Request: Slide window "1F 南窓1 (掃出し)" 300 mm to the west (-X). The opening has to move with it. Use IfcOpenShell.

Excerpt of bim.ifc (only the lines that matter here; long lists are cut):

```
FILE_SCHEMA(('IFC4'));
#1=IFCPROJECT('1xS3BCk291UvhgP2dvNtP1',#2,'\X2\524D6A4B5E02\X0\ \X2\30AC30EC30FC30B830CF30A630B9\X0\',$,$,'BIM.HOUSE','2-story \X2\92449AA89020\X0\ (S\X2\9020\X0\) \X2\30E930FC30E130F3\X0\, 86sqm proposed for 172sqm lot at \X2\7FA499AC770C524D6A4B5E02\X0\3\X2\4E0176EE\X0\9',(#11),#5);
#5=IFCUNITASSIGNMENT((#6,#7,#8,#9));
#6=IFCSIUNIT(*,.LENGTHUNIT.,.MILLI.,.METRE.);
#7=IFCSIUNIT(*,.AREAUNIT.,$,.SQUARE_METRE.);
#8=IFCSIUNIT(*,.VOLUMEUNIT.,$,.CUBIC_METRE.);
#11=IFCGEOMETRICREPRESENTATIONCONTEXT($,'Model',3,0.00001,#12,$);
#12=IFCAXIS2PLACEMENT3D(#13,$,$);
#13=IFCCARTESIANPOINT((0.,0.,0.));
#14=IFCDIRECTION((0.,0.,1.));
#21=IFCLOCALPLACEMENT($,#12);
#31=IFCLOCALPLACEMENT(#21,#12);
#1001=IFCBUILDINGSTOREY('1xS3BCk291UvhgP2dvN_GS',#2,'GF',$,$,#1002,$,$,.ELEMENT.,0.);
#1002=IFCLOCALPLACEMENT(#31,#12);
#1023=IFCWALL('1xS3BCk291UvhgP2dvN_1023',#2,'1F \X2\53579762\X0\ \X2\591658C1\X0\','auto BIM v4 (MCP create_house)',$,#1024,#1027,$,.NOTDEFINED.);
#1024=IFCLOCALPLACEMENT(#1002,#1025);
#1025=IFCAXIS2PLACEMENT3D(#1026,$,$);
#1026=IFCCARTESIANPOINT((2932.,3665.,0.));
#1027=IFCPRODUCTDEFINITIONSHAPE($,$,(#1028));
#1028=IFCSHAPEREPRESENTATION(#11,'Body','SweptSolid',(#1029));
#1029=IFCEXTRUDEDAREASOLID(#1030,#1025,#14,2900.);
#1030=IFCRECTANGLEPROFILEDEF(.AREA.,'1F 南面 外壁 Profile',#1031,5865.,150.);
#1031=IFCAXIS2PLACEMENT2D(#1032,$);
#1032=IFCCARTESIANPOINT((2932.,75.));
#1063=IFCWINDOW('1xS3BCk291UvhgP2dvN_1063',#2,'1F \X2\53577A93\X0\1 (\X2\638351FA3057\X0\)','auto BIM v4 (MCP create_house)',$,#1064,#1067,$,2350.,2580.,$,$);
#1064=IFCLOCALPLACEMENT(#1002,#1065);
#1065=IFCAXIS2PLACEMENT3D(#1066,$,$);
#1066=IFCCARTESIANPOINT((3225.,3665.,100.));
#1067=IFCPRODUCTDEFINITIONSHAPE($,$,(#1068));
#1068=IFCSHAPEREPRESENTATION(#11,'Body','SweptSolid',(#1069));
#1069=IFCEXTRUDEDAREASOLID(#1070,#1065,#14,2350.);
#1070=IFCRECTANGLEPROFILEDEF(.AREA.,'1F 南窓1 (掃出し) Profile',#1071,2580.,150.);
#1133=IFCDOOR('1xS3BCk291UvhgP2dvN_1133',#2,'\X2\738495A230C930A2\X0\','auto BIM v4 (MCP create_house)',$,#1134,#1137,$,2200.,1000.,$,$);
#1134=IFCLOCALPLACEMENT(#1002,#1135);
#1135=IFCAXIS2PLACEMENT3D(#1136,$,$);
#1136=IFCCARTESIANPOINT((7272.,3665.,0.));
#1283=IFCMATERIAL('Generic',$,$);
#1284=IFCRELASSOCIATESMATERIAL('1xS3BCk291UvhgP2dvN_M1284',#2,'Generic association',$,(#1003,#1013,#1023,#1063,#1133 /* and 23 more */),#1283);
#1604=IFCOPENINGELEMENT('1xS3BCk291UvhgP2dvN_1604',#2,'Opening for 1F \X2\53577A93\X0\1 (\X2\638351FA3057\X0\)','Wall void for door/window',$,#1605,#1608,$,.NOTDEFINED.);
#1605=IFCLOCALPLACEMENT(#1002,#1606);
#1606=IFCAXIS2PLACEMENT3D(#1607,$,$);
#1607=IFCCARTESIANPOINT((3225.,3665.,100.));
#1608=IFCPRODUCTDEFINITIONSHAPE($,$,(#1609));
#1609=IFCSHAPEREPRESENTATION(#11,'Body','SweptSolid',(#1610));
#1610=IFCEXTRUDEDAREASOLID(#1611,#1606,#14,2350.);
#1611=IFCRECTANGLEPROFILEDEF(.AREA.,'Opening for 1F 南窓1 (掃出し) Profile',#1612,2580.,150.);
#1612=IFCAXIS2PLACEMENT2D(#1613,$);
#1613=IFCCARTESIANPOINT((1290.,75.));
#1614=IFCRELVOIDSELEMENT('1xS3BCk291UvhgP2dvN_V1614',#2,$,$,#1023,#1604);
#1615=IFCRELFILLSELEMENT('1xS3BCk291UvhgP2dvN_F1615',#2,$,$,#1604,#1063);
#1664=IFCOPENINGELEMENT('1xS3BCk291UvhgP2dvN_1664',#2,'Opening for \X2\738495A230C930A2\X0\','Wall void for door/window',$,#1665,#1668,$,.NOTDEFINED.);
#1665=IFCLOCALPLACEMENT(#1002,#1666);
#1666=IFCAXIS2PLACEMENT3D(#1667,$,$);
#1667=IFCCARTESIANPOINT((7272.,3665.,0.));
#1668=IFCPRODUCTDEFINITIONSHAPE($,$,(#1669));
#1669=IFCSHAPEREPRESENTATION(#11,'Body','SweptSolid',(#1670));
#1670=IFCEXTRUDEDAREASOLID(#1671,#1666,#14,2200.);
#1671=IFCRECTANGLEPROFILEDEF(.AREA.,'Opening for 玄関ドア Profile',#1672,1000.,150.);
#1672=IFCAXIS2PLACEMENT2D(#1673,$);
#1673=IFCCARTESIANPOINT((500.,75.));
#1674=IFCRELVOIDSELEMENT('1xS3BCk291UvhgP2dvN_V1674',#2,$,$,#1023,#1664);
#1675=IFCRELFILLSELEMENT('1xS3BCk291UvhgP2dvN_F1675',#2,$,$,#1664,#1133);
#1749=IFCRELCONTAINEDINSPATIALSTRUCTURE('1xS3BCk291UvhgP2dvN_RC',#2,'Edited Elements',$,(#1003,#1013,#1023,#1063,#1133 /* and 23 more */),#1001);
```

```python
import ifcopenshell
import ifcopenshell.api.geometry
import ifcopenshell.util.placement

model = ifcopenshell.open("bim.ifc")

window = model.by_guid("1xS3BCk291UvhgP2dvN_1063")
opening = window.FillsVoids[0].RelatingOpeningElement
wall = opening.VoidsElements[0].RelatingBuildingElement

wall_matrix = ifcopenshell.util.placement.get_local_placement(wall.ObjectPlacement)
shift = wall_matrix[:3, 0] * -300.0
before = ifcopenshell.util.placement.get_local_placement(window.ObjectPlacement)[:3, 3].copy()

# The window is not placed relative to its opening, so move both.
for product in (opening, window):
    matrix = ifcopenshell.util.placement.get_local_placement(product.ObjectPlacement)
    matrix[:3, 3] += shift
    ifcopenshell.api.geometry.edit_object_placement(model, product=product, matrix=matrix, is_si=False)

after = ifcopenshell.util.placement.get_local_placement(window.ObjectPlacement)[:3, 3]
print("window moved by", (after - before).round(3) + 0.0)

model.write("bim_updated.ifc")
```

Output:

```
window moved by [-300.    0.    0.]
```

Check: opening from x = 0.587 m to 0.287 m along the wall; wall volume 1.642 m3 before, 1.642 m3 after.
